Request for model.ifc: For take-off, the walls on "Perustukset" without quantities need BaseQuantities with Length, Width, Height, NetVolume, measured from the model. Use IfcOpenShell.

First a look at what the model holds.

```python
import ifcopenshell
import ifcopenshell.util.element
import ifcopenshell.util.unit

model = ifcopenshell.open("model.ifc")
print(model.schema)
for unit_type in ("LENGTHUNIT", "AREAUNIT", "VOLUMEUNIT"):
    print(unit_type, ifcopenshell.util.unit.calculate_unit_scale(model, unit_type))
storey = next(s for s in model.by_type("IfcBuildingStorey") if s.Name == "Perustukset")
walls = [e for e in ifcopenshell.util.element.get_decomposition(storey) if e.is_a("IfcWall")]
for e in sorted(walls, key=lambda e: e.id()):
    print(e.id(), e.is_a(), e.Name, list(ifcopenshell.util.element.get_psets(e, qtos_only=True)), sep=" | ")
```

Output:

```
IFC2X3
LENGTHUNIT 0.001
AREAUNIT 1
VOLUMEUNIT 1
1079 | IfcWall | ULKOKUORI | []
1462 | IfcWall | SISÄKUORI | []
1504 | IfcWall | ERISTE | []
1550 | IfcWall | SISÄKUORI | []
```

```python
import ifcopenshell
import ifcopenshell.api.pset
import ifcopenshell.geom
import ifcopenshell.util.element
import ifcopenshell.util.shape
import ifcopenshell.util.unit

model = ifcopenshell.open("model.ifc")
unit_scale = ifcopenshell.util.unit.calculate_unit_scale(model)
volume_scale = ifcopenshell.util.unit.calculate_unit_scale(model, "VOLUMEUNIT")
settings = ifcopenshell.geom.settings()

storey = next(s for s in model.by_type("IfcBuildingStorey") if s.Name == "Perustukset")
walls = [e for e in ifcopenshell.util.element.get_decomposition(storey) if e.is_a("IfcWall")]

for e in sorted(walls, key=lambda e: e.id()):
    if ifcopenshell.util.element.get_psets(e, qtos_only=True, should_inherit=False):
        continue
    # Geometry comes back in metres, in the element's own axes.
    shape = ifcopenshell.geom.create_shape(settings, e)
    values = {
        "Length": ifcopenshell.util.shape.get_x(shape.geometry) / unit_scale,
        "Width": ifcopenshell.util.shape.get_y(shape.geometry) / unit_scale,
        "Height": ifcopenshell.util.shape.get_z(shape.geometry) / unit_scale,
        "NetVolume": ifcopenshell.util.shape.get_volume(shape.geometry) / volume_scale,
    }
    qto = ifcopenshell.api.pset.add_qto(model, product=e, name="BaseQuantities")
    ifcopenshell.api.pset.edit_qto(model, qto=qto, properties=values)
    print(e.id(), {k: round(v, 3) for k, v in values.items()})

model.write("model_v2.ifc")
```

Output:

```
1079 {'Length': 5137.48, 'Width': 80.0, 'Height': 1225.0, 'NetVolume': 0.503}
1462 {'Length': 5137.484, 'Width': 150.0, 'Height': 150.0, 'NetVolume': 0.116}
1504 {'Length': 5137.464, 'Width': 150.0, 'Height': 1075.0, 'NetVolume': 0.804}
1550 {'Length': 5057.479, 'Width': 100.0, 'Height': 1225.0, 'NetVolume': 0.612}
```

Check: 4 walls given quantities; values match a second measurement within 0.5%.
